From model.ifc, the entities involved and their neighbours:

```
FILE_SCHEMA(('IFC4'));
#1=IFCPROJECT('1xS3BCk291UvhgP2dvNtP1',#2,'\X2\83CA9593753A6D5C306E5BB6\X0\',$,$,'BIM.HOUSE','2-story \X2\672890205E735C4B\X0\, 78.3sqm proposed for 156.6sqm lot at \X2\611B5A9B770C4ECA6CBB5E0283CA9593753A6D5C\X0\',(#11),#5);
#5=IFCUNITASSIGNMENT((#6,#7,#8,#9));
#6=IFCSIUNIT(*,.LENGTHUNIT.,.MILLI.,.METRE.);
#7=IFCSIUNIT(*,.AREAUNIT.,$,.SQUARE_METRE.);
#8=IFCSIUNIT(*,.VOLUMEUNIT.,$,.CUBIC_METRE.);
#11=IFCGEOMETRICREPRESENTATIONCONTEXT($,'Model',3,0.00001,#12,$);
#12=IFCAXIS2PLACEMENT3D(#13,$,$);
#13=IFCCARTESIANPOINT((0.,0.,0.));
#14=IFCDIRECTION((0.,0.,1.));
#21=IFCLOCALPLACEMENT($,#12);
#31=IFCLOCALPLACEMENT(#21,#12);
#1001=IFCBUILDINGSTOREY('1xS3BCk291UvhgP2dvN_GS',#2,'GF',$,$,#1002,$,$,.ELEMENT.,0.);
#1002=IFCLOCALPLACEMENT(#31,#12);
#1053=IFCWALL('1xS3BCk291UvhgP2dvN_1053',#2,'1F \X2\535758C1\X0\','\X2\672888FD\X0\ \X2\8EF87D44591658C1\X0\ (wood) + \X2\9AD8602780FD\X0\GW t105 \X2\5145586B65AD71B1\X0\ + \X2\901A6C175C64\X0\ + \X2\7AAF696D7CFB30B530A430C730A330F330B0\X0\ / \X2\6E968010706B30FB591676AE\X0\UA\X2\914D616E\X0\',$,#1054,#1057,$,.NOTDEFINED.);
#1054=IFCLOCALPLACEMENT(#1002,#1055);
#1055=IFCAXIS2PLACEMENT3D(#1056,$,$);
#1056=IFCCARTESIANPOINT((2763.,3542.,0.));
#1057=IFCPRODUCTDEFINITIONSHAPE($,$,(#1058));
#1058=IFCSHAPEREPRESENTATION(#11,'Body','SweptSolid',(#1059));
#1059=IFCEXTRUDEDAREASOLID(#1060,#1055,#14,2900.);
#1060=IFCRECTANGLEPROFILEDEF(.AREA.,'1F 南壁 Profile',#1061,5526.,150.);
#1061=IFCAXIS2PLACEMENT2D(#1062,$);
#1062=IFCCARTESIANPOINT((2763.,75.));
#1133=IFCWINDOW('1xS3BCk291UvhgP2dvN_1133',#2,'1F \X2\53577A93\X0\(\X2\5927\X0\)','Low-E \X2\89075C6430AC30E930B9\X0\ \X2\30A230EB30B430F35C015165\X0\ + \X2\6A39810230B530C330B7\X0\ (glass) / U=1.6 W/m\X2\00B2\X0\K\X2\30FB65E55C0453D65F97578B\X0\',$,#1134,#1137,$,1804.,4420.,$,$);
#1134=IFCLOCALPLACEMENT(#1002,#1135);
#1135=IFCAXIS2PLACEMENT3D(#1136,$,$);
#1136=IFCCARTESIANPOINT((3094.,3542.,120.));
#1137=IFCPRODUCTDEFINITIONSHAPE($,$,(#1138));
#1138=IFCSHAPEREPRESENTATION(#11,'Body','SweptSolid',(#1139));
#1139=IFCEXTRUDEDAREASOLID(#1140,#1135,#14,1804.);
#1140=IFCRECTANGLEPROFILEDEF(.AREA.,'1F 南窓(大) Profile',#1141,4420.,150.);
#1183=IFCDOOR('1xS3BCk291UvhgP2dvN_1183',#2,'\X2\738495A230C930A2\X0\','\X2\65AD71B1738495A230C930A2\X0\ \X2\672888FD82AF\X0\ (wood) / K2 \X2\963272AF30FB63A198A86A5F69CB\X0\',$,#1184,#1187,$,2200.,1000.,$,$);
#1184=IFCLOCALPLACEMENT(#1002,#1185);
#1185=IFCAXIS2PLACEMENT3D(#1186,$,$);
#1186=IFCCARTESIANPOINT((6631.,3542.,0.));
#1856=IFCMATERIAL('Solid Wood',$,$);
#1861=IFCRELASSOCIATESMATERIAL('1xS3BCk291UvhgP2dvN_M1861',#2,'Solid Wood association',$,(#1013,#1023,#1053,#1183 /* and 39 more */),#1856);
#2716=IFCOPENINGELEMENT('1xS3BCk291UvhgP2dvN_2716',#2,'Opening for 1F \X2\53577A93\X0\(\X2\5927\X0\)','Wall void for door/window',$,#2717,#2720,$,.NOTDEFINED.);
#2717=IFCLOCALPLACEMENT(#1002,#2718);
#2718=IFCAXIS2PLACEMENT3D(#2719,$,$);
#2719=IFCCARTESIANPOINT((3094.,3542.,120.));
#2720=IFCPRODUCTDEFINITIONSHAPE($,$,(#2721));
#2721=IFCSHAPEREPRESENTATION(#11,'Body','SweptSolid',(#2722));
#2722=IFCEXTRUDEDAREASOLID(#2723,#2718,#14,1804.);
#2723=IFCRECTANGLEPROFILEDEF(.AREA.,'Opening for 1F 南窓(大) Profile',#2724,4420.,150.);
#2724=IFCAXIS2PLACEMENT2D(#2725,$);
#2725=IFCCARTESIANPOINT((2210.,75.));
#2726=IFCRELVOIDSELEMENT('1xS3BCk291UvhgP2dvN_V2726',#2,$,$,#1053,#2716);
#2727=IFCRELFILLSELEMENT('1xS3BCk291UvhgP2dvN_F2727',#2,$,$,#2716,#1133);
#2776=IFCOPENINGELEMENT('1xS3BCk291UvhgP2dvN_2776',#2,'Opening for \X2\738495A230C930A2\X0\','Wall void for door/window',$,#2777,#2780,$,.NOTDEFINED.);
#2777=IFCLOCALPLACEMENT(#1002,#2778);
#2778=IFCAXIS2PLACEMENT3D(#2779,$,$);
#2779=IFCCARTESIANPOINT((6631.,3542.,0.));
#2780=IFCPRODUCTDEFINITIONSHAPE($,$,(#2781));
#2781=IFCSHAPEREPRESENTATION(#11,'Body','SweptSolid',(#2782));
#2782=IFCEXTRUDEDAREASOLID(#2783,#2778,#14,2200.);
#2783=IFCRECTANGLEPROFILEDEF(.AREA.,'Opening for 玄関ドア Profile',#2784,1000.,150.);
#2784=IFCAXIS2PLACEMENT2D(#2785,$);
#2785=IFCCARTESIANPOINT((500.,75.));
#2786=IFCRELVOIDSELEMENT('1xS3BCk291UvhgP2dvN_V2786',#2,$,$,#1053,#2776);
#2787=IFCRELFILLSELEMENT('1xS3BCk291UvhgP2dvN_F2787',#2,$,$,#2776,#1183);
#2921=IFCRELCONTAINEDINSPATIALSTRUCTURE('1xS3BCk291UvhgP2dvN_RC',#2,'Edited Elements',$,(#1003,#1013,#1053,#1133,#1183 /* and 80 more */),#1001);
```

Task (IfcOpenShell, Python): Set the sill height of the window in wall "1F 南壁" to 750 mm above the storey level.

```python
import numpy as np
import ifcopenshell
import ifcopenshell.api.geometry
import ifcopenshell.geom
import ifcopenshell.util.element
import ifcopenshell.util.placement
import ifcopenshell.util.shape
import ifcopenshell.util.unit

model = ifcopenshell.open("model.ifc")
unit_scale = ifcopenshell.util.unit.calculate_unit_scale(model)

window = model.by_guid("1xS3BCk291UvhgP2dvN_1133")
opening = window.FillsVoids[0].RelatingOpeningElement
storey = ifcopenshell.util.element.get_container(window, ifc_class="IfcBuildingStorey")
level = ifcopenshell.util.placement.get_local_placement(storey.ObjectPlacement)[2, 3]

# The opening's origin need not be at the sill, so measure its lowest point.
shape = ifcopenshell.geom.create_shape(ifcopenshell.geom.settings(), opening)
bottom = ifcopenshell.util.shape.get_shape_bottom_elevation(shape, shape.geometry) / unit_scale
dz = level + 0.75 / unit_scale - bottom

shift = np.array([0.0, 0.0, dz])
# The window is not placed relative to its opening, so move both.
for product in (opening, window):
    matrix = ifcopenshell.util.placement.get_local_placement(product.ObjectPlacement)
    matrix[:3, 3] += shift
    ifcopenshell.api.geometry.edit_object_placement(model, product=product, matrix=matrix, is_si=False)

print(f"moved by {dz * unit_scale:+.3f} m")

model.write("model_updated.ifc")
```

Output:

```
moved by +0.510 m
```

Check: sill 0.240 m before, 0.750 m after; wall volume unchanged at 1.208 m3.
